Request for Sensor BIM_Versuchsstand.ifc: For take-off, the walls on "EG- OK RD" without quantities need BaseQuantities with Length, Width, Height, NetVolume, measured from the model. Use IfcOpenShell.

First a look at what the model holds.

```python
import ifcopenshell
import ifcopenshell.util.element
import ifcopenshell.util.unit

model = ifcopenshell.open("Sensor BIM_Versuchsstand.ifc")
print(model.schema)
for unit_type in ("LENGTHUNIT", "AREAUNIT", "VOLUMEUNIT"):
    print(unit_type, ifcopenshell.util.unit.calculate_unit_scale(model, unit_type))
storey = next(s for s in model.by_type("IfcBuildingStorey") if s.Name == "EG- OK RD")
walls = [e for e in ifcopenshell.util.element.get_decomposition(storey) if e.is_a("IfcWall")]
for e in sorted(walls, key=lambda e: e.id()):
    print(e.id(), e.is_a(), e.Name, list(ifcopenshell.util.element.get_psets(e, qtos_only=True)), sep=" | ")
```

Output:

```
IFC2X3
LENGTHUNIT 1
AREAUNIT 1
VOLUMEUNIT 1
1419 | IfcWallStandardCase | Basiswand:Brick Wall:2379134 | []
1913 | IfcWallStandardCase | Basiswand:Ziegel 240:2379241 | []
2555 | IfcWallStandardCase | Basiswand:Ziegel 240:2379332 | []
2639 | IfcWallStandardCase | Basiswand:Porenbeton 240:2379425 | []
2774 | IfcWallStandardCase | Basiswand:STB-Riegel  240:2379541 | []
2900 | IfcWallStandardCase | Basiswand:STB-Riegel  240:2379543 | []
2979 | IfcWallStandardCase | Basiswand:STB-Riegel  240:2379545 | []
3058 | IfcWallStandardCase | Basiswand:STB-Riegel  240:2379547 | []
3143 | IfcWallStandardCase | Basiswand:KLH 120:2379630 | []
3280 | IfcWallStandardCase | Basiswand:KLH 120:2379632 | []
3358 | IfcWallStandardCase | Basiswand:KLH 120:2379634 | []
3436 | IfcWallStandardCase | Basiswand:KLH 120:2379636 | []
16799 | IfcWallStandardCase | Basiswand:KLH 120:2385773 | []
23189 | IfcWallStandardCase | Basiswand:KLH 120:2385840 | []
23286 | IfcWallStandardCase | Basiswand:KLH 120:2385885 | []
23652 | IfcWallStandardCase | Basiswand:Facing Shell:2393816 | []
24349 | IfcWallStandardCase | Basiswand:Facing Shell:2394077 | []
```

```python
import ifcopenshell
import ifcopenshell.api.pset
import ifcopenshell.geom
import ifcopenshell.util.element
import ifcopenshell.util.shape
import ifcopenshell.util.unit

model = ifcopenshell.open("Sensor BIM_Versuchsstand.ifc")
unit_scale = ifcopenshell.util.unit.calculate_unit_scale(model)
volume_scale = ifcopenshell.util.unit.calculate_unit_scale(model, "VOLUMEUNIT")
settings = ifcopenshell.geom.settings()

storey = next(s for s in model.by_type("IfcBuildingStorey") if s.Name == "EG- OK RD")
walls = [e for e in ifcopenshell.util.element.get_decomposition(storey) if e.is_a("IfcWall")]

for e in sorted(walls, key=lambda e: e.id()):
    if ifcopenshell.util.element.get_psets(e, qtos_only=True, should_inherit=False):
        continue
    # Geometry comes back in metres, in the element's own axes.
    shape = ifcopenshell.geom.create_shape(settings, e)
    values = {
        "Length": ifcopenshell.util.shape.get_x(shape.geometry) / unit_scale,
        "Width": ifcopenshell.util.shape.get_y(shape.geometry) / unit_scale,
        "Height": ifcopenshell.util.shape.get_z(shape.geometry) / unit_scale,
        "NetVolume": ifcopenshell.util.shape.get_volume(shape.geometry) / volume_scale,
    }
    qto = ifcopenshell.api.pset.add_qto(model, product=e, name="BaseQuantities")
    ifcopenshell.api.pset.edit_qto(model, qto=qto, properties=values)
    print(e.id(), {k: round(v, 3) for k, v in values.items()})

model.write("Sensor BIM_Versuchsstand_rev.ifc")
```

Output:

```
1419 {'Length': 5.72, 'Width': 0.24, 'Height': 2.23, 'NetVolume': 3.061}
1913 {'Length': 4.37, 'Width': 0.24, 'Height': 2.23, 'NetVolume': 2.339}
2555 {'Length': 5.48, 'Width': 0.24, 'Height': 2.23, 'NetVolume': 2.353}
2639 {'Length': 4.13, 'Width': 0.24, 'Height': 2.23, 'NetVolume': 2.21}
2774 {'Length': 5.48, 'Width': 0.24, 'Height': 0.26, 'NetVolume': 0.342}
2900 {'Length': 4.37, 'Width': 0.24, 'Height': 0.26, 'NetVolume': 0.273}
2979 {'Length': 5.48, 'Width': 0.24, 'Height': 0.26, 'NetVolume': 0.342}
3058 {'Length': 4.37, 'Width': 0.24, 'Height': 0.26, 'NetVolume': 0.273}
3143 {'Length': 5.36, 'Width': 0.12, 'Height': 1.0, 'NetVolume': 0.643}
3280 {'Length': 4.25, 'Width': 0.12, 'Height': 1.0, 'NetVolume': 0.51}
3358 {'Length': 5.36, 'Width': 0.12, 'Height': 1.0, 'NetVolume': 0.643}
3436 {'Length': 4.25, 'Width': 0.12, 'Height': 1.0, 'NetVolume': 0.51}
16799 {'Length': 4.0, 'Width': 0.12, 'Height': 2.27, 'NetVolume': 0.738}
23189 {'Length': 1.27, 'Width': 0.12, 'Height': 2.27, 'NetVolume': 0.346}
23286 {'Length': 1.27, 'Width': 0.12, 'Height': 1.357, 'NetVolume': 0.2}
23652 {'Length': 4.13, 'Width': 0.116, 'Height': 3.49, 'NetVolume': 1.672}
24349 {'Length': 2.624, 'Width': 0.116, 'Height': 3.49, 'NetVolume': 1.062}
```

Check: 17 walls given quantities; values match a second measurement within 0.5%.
